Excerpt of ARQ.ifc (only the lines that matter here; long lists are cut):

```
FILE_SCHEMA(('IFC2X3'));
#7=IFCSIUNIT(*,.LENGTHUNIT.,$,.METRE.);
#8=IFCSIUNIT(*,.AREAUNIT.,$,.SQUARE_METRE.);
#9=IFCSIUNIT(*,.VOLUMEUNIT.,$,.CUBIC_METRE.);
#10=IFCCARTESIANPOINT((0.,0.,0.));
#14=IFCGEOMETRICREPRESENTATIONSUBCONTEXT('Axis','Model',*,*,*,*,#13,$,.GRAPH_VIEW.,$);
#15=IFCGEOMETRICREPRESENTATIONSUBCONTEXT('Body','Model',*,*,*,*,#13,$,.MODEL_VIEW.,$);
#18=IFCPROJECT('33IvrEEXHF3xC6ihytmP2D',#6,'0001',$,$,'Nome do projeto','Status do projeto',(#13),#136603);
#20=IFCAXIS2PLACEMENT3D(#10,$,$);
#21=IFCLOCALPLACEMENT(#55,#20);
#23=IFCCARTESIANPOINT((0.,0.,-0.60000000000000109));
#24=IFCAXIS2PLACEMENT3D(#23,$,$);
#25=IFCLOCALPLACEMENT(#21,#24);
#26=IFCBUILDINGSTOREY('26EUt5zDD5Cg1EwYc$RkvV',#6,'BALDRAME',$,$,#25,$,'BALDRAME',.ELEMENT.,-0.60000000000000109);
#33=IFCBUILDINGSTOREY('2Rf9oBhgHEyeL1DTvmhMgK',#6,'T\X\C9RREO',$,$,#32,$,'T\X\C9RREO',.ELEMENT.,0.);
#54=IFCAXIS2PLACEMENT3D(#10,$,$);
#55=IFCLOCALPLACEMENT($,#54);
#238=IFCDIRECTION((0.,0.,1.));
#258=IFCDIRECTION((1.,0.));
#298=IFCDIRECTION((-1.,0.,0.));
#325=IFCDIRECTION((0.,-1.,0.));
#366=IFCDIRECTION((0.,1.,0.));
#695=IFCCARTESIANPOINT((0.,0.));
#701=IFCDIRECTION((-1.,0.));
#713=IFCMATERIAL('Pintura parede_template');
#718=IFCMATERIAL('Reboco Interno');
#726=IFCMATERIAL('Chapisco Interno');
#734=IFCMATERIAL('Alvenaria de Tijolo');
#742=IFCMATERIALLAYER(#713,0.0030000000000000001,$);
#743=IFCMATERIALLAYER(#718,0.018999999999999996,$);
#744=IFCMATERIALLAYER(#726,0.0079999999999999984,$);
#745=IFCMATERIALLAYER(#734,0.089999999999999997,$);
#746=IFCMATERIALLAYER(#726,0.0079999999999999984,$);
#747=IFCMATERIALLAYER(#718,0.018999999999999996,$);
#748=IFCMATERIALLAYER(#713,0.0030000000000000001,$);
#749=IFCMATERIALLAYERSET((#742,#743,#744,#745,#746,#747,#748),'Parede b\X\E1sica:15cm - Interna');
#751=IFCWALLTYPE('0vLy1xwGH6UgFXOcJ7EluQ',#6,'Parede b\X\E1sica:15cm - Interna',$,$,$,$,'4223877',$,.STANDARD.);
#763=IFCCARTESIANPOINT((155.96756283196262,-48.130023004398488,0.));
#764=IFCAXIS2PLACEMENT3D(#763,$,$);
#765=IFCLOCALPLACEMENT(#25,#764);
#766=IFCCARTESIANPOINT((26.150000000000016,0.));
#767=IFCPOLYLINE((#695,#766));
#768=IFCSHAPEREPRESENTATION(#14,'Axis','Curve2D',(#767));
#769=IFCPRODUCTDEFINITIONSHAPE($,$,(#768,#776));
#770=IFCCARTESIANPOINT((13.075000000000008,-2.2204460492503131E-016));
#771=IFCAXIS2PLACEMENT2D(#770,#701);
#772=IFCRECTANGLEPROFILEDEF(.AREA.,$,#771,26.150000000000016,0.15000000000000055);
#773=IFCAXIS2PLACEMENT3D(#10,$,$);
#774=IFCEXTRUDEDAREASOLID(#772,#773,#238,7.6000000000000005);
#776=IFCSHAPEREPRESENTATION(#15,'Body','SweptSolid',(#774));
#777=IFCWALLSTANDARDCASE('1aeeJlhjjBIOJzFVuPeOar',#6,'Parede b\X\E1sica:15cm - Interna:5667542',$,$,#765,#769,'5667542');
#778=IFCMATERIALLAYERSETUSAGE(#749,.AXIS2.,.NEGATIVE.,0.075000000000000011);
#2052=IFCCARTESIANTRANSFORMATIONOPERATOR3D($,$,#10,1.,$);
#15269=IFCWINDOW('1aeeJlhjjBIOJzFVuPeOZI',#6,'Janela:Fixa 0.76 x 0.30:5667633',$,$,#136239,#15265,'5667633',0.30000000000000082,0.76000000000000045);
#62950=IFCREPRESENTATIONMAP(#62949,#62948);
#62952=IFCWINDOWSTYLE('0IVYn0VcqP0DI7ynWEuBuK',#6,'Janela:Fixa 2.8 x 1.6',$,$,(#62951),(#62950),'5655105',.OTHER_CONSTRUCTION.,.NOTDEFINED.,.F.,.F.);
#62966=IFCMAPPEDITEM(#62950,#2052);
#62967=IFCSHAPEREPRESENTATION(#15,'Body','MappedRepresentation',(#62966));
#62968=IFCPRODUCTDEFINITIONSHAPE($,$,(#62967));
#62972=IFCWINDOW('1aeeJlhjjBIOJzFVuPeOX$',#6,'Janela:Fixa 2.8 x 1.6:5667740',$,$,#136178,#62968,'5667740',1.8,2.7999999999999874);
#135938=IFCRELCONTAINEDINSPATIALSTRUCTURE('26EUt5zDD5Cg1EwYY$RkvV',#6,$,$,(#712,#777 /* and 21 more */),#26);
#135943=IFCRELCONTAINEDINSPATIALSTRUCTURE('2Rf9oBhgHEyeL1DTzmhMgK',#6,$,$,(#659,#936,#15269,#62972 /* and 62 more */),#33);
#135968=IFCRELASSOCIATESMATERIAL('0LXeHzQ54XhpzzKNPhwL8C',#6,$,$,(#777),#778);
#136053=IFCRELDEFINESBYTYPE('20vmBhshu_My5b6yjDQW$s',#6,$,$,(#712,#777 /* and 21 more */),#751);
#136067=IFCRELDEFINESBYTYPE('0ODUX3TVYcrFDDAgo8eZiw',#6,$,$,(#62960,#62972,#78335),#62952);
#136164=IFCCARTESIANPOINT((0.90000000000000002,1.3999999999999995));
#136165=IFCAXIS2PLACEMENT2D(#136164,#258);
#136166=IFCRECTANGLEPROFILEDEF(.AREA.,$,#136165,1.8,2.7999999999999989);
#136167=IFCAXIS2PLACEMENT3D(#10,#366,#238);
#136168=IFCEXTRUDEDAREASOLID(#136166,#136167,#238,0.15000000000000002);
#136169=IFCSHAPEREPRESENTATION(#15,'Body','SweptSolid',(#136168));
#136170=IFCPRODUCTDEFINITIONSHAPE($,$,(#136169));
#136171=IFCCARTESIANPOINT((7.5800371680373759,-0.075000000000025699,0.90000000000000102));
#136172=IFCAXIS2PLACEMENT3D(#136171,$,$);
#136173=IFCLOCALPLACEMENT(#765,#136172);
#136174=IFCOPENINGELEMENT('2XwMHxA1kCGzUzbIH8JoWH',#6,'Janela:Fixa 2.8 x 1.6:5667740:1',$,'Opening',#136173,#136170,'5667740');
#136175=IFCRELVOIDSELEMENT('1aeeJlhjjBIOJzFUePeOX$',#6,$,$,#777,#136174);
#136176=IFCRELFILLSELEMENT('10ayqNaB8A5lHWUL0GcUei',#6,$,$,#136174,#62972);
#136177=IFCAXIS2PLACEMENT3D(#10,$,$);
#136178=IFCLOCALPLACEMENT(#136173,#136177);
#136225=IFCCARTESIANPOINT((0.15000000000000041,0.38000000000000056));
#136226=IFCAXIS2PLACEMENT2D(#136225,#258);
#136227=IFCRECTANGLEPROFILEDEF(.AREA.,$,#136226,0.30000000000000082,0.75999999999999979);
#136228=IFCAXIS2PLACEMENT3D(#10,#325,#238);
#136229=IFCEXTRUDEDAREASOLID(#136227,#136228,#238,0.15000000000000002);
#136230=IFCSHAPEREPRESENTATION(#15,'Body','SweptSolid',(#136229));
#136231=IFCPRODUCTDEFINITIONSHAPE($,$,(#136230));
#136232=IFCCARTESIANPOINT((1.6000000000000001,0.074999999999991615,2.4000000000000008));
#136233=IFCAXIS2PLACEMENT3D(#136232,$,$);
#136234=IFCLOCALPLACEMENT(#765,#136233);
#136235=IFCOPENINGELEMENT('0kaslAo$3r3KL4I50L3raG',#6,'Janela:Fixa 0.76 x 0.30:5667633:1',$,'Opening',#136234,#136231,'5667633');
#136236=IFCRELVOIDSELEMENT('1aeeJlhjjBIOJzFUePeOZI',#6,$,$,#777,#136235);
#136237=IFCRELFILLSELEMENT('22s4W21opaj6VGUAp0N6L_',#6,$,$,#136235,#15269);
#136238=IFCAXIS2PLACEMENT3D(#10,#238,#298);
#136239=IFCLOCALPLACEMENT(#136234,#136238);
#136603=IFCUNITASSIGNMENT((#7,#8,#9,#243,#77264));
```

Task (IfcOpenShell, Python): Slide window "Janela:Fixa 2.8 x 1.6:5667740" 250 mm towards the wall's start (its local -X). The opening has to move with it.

```python
import ifcopenshell
import ifcopenshell.api.geometry
import ifcopenshell.util.placement
import ifcopenshell.util.unit

model = ifcopenshell.open("ARQ.ifc")
unit_scale = ifcopenshell.util.unit.calculate_unit_scale(model)

window = model.by_id(62972)
opening = window.FillsVoids[0].RelatingOpeningElement
wall = opening.VoidsElements[0].RelatingBuildingElement

wall_matrix = ifcopenshell.util.placement.get_local_placement(wall.ObjectPlacement)
shift = wall_matrix[:3, 0] * -0.25 / unit_scale
before = ifcopenshell.util.placement.get_local_placement(window.ObjectPlacement)[:3, 3].copy()

# The window is placed relative to its opening, so it follows when the opening moves.
matrix = ifcopenshell.util.placement.get_local_placement(opening.ObjectPlacement)
matrix[:3, 3] += shift
ifcopenshell.api.geometry.edit_object_placement(
    model, product=opening, matrix=matrix, is_si=False, should_transform_children=True
)

after = ifcopenshell.util.placement.get_local_placement(window.ObjectPlacement)[:3, 3]
print("window moved by", (after - before).round(3) + 0.0)

model.write("ARQ_v2.ifc")
```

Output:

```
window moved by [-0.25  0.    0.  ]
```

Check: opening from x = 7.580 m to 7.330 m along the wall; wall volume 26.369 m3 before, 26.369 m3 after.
